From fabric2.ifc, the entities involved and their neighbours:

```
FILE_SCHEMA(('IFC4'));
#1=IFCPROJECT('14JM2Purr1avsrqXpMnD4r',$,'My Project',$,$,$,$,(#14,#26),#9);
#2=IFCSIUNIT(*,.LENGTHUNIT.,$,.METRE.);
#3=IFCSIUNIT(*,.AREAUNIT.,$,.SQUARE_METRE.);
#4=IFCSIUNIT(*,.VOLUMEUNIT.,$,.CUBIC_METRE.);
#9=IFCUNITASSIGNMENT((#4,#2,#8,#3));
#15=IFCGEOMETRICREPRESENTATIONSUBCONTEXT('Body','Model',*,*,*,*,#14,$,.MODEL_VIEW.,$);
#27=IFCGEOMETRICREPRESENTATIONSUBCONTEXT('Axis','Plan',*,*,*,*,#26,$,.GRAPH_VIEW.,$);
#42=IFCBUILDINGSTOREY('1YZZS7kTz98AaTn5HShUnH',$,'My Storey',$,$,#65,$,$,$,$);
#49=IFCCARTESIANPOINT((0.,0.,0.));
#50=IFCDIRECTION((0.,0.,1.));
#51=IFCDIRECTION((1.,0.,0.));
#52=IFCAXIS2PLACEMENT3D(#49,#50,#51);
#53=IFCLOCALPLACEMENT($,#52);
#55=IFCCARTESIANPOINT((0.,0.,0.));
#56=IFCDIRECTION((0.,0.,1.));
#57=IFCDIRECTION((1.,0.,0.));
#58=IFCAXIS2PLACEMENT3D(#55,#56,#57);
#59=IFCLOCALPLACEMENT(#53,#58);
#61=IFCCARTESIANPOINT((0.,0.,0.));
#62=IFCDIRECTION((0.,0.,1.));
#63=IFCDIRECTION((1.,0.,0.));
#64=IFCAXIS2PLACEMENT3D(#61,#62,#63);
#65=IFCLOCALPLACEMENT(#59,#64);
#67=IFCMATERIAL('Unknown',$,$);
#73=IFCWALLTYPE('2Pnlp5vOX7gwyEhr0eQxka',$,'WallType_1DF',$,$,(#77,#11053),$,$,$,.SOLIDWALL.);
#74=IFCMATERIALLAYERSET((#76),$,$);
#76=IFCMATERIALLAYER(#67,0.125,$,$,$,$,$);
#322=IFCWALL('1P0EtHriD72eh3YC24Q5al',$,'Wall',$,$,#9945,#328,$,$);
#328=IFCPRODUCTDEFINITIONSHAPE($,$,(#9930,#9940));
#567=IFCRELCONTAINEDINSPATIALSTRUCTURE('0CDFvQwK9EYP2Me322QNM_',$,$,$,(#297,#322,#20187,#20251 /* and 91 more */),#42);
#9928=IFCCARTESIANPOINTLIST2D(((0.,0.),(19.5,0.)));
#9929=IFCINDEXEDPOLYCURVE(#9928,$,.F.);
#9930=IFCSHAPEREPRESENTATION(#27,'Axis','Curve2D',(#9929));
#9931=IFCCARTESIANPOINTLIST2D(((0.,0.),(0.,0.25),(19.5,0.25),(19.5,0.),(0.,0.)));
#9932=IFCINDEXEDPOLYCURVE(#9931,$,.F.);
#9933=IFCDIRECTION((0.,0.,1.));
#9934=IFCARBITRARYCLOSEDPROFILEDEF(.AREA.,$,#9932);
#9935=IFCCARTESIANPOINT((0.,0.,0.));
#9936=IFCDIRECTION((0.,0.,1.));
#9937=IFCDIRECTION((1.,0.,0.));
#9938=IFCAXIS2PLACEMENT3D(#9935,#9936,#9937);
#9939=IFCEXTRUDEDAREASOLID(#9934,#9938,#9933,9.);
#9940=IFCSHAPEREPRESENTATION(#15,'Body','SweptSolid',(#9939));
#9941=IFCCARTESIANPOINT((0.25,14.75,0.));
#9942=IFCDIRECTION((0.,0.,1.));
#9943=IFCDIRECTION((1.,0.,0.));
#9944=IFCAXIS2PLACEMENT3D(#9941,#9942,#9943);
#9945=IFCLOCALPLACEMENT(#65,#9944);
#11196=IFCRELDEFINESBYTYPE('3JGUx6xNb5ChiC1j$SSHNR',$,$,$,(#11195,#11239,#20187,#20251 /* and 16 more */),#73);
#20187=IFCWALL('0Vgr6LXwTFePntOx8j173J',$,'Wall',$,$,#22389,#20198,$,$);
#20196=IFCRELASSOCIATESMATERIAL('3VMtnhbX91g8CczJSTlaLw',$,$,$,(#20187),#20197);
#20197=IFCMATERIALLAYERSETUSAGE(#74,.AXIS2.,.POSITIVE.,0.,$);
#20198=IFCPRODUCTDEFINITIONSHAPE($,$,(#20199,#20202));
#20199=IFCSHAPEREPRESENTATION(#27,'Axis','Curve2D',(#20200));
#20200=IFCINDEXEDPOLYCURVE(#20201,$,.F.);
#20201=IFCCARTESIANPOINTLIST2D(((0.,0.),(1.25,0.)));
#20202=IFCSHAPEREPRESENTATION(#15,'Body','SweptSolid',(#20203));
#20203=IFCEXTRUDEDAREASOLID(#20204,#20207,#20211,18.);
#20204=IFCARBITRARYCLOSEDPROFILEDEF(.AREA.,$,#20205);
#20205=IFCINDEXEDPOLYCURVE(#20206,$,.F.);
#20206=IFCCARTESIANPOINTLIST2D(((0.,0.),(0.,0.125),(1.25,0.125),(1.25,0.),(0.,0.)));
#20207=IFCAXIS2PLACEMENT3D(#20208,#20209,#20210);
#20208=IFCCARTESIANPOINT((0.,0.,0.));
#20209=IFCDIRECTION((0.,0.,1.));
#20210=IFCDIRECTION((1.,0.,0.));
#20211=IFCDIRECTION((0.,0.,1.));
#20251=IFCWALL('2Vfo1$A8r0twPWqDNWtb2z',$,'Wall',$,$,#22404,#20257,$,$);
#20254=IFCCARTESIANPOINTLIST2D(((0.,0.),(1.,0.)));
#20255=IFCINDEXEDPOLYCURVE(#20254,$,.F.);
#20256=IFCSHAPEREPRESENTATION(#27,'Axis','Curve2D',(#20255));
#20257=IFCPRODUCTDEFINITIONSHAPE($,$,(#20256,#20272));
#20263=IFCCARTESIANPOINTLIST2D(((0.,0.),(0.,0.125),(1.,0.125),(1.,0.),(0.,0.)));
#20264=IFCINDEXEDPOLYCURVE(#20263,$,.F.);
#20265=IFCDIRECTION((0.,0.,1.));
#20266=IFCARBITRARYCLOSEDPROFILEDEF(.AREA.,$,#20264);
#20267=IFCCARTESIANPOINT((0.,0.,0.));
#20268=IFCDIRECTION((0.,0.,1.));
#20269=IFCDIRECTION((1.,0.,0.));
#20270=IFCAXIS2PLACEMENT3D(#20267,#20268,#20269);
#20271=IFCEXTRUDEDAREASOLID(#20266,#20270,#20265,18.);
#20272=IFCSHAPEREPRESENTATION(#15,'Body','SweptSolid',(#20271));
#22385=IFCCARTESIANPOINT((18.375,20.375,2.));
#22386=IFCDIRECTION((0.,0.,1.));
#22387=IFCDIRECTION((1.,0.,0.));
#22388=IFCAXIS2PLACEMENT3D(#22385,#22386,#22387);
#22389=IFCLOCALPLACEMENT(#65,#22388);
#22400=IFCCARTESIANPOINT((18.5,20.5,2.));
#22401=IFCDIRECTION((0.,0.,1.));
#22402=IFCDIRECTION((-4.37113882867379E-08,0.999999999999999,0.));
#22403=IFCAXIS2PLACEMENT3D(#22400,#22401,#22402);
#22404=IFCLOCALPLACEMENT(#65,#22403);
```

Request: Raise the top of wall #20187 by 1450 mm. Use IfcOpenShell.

```python
import ifcopenshell
import ifcopenshell.geom
import ifcopenshell.util.representation
import ifcopenshell.util.shape
import ifcopenshell.util.unit

model = ifcopenshell.open("fabric2.ifc")
unit_scale = ifcopenshell.util.unit.calculate_unit_scale(model)
settings = ifcopenshell.geom.settings()


def volume(element):
    """Net volume in cubic metres, openings subtracted."""
    shape = ifcopenshell.geom.create_shape(settings, element)
    return ifcopenshell.util.shape.get_volume(shape.geometry)


wall = model.by_guid("0Vgr6LXwTFePntOx8j173J")
before = volume(wall)

body = ifcopenshell.util.representation.get_representation(wall, "Model", "Body")
solid = body.Items[0]
old_height = solid.Depth
solid.Depth += 1.45 / unit_scale
after = volume(wall)

print(f"height {old_height:g} -> {solid.Depth:g}, volume {before:.3f} -> {after:.3f} m3")

model.write("fabric2_updated.ifc")
```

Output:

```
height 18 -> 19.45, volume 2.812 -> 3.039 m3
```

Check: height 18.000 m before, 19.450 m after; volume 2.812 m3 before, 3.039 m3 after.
